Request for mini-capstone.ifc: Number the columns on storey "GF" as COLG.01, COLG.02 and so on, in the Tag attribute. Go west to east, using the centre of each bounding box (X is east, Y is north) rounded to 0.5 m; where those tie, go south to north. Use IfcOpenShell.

First a look at what the model holds.

```python
import ifcopenshell
import ifcopenshell.util.element
import ifcopenshell.util.placement

model = ifcopenshell.open("mini-capstone.ifc")
print(model.schema)
storey = next(s for s in model.by_type("IfcBuildingStorey") if s.Name == "GF")
columns = [e for e in ifcopenshell.util.element.get_decomposition(storey) if e.is_a("IfcColumn")]
for e in sorted(columns, key=lambda e: e.id()):
    origin = ifcopenshell.util.placement.get_local_placement(e.ObjectPlacement)[:3, 3]
    print(e.id(), e.Tag, e.Name, origin.round(2) + 0.0, sep=" | ")
```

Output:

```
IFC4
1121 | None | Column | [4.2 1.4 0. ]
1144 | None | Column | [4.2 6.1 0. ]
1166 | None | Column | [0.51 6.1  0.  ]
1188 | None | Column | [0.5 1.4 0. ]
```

```python
import ifcopenshell
import ifcopenshell.geom
import ifcopenshell.util.element
import ifcopenshell.util.shape

model = ifcopenshell.open("mini-capstone.ifc")
settings = ifcopenshell.geom.settings()
settings.set("use-world-coords", True)


def centre(element):
    shape = ifcopenshell.geom.create_shape(settings, element)
    return ifcopenshell.util.shape.get_bbox_centroid(shape.geometry)


storey = next(s for s in model.by_type("IfcBuildingStorey") if s.Name == "GF")
columns = [e for e in ifcopenshell.util.element.get_decomposition(storey) if e.is_a("IfcColumn")]

# Insertion points can sit at a corner or the storey origin, so sort by the geometry (in metres).
centres = {e: centre(e) for e in columns}
columns.sort(key=lambda e: (round(centres[e][0] / 0.5), centres[e][1]))

for i, e in enumerate(columns, start=1):
    number = f"COLG.{i:02d}"
    e.Tag = number
    print(e.id(), number)

model.write("mini-capstone_edited.ifc")
```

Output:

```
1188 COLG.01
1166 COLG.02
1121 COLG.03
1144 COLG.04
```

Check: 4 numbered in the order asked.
